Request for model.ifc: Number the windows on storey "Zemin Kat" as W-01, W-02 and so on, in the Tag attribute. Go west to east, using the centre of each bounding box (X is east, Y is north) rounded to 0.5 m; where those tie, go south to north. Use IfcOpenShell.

First a look at what the model holds.

```python
import ifcopenshell
import ifcopenshell.util.element
import ifcopenshell.util.placement

model = ifcopenshell.open("model.ifc")
print(model.schema)
storey = next(s for s in model.by_type("IfcBuildingStorey") if s.Name == "Zemin Kat")
windows = [e for e in ifcopenshell.util.element.get_decomposition(storey) if e.is_a("IfcWindow")]
for e in sorted(windows, key=lambda e: e.id()):
    origin = ifcopenshell.util.placement.get_local_placement(e.ObjectPlacement)[:3, 3]
    print(e.id(), e.Tag, e.Name, origin.round(2) + 0.0, sep=" | ")
```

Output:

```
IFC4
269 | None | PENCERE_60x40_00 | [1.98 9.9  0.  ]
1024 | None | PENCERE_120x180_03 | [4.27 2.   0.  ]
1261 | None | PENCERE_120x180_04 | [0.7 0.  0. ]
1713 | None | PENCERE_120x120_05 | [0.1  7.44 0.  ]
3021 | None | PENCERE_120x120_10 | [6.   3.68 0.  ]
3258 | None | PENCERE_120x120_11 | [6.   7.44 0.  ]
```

```python
import ifcopenshell
import ifcopenshell.geom
import ifcopenshell.util.element
import ifcopenshell.util.shape

model = ifcopenshell.open("model.ifc")
settings = ifcopenshell.geom.settings()
settings.set("use-world-coords", True)


def centre(element):
    shape = ifcopenshell.geom.create_shape(settings, element)
    return ifcopenshell.util.shape.get_bbox_centroid(shape.geometry)


storey = next(s for s in model.by_type("IfcBuildingStorey") if s.Name == "Zemin Kat")
windows = [e for e in ifcopenshell.util.element.get_decomposition(storey) if e.is_a("IfcWindow")]

# Insertion points can sit at a corner or the storey origin, so sort by the geometry (in metres).
centres = {e: centre(e) for e in windows}
windows.sort(key=lambda e: (round(centres[e][0] / 0.5), centres[e][1]))

for i, e in enumerate(windows, start=1):
    number = f"W-{i:02d}"
    e.Tag = number
    print(e.id(), number)

model.write("model_updated.ifc")
```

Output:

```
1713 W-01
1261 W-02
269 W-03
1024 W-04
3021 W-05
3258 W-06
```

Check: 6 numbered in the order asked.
